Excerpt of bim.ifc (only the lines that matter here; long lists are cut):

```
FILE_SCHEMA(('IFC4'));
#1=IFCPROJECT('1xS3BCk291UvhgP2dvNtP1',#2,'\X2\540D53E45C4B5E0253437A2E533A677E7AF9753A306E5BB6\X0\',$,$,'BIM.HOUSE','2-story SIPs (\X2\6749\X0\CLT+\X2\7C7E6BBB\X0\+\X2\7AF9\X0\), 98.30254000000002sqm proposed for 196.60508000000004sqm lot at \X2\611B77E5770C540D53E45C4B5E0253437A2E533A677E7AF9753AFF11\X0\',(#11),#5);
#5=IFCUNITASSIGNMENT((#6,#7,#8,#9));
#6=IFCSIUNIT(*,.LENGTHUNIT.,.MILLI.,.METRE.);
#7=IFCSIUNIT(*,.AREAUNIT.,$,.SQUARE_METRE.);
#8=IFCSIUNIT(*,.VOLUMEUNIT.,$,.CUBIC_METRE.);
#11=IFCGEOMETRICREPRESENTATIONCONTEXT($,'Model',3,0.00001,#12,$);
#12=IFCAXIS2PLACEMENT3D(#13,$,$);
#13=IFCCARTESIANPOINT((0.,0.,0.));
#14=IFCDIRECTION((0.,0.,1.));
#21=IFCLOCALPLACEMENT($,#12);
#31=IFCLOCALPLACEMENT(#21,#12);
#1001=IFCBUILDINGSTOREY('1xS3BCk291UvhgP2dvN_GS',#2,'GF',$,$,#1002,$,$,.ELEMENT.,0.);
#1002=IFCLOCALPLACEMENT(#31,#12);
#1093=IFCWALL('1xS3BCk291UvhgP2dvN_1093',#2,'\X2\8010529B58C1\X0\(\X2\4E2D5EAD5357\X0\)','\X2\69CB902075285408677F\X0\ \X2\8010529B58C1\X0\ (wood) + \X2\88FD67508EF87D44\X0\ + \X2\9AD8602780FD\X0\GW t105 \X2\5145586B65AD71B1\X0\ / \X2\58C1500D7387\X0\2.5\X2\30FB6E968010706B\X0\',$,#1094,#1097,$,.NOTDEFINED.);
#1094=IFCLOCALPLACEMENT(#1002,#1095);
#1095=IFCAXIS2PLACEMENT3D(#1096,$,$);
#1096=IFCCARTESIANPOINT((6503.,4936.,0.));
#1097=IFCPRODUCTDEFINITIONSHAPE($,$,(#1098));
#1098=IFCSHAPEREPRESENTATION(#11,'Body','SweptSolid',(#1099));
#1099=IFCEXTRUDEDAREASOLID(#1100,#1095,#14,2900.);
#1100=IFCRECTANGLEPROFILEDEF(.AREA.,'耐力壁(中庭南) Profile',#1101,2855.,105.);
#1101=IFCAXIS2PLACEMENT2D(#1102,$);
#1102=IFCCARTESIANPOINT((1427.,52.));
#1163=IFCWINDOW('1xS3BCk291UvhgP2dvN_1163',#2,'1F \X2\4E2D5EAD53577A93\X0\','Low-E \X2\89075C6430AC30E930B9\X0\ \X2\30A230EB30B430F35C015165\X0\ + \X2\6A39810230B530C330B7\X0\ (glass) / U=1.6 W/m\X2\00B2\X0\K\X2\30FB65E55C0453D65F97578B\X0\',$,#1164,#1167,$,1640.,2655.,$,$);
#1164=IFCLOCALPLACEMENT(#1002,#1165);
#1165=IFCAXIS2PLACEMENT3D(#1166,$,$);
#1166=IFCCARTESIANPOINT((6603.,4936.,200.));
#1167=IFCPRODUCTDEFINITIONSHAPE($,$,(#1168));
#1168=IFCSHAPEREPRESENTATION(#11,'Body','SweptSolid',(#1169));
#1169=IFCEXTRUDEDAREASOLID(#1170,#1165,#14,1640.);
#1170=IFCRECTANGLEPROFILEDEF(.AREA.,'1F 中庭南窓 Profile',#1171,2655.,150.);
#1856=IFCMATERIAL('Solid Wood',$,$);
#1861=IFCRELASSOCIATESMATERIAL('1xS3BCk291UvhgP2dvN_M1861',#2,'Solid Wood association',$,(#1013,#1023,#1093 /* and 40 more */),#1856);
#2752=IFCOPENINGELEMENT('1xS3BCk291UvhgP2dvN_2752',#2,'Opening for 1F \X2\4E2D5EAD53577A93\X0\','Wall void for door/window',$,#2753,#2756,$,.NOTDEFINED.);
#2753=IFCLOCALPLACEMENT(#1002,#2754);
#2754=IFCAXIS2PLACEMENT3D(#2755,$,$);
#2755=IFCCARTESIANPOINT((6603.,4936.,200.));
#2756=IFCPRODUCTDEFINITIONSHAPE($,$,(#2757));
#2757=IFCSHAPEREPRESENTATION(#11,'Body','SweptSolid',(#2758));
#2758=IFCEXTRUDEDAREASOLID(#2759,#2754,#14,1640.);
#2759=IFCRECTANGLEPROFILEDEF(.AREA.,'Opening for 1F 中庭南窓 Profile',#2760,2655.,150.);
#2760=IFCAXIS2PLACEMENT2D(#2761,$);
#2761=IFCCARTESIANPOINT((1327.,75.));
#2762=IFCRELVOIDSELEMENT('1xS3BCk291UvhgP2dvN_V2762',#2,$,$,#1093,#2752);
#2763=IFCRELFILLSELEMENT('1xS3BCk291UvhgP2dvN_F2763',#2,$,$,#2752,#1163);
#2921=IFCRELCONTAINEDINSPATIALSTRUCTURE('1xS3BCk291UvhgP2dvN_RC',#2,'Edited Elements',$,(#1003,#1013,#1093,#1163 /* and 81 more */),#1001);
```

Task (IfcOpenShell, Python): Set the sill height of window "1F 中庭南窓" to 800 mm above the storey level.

```python
import numpy as np
import ifcopenshell
import ifcopenshell.api.geometry
import ifcopenshell.geom
import ifcopenshell.util.element
import ifcopenshell.util.placement
import ifcopenshell.util.shape
import ifcopenshell.util.unit

model = ifcopenshell.open("bim.ifc")
unit_scale = ifcopenshell.util.unit.calculate_unit_scale(model)

window = model.by_guid("1xS3BCk291UvhgP2dvN_1163")
opening = window.FillsVoids[0].RelatingOpeningElement
storey = ifcopenshell.util.element.get_container(window, ifc_class="IfcBuildingStorey")
level = ifcopenshell.util.placement.get_local_placement(storey.ObjectPlacement)[2, 3]

# The opening's origin need not be at the sill, so measure its lowest point.
shape = ifcopenshell.geom.create_shape(ifcopenshell.geom.settings(), opening)
bottom = ifcopenshell.util.shape.get_shape_bottom_elevation(shape, shape.geometry) / unit_scale
dz = level + 0.8 / unit_scale - bottom

shift = np.array([0.0, 0.0, dz])
# The window is not placed relative to its opening, so move both.
for product in (opening, window):
    matrix = ifcopenshell.util.placement.get_local_placement(product.ObjectPlacement)
    matrix[:3, 3] += shift
    ifcopenshell.api.geometry.edit_object_placement(model, product=product, matrix=matrix, is_si=False)

print(f"moved by {dz * unit_scale:+.3f} m")

model.write("bim_updated.ifc")
```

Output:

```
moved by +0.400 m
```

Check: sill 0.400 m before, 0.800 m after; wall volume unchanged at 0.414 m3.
